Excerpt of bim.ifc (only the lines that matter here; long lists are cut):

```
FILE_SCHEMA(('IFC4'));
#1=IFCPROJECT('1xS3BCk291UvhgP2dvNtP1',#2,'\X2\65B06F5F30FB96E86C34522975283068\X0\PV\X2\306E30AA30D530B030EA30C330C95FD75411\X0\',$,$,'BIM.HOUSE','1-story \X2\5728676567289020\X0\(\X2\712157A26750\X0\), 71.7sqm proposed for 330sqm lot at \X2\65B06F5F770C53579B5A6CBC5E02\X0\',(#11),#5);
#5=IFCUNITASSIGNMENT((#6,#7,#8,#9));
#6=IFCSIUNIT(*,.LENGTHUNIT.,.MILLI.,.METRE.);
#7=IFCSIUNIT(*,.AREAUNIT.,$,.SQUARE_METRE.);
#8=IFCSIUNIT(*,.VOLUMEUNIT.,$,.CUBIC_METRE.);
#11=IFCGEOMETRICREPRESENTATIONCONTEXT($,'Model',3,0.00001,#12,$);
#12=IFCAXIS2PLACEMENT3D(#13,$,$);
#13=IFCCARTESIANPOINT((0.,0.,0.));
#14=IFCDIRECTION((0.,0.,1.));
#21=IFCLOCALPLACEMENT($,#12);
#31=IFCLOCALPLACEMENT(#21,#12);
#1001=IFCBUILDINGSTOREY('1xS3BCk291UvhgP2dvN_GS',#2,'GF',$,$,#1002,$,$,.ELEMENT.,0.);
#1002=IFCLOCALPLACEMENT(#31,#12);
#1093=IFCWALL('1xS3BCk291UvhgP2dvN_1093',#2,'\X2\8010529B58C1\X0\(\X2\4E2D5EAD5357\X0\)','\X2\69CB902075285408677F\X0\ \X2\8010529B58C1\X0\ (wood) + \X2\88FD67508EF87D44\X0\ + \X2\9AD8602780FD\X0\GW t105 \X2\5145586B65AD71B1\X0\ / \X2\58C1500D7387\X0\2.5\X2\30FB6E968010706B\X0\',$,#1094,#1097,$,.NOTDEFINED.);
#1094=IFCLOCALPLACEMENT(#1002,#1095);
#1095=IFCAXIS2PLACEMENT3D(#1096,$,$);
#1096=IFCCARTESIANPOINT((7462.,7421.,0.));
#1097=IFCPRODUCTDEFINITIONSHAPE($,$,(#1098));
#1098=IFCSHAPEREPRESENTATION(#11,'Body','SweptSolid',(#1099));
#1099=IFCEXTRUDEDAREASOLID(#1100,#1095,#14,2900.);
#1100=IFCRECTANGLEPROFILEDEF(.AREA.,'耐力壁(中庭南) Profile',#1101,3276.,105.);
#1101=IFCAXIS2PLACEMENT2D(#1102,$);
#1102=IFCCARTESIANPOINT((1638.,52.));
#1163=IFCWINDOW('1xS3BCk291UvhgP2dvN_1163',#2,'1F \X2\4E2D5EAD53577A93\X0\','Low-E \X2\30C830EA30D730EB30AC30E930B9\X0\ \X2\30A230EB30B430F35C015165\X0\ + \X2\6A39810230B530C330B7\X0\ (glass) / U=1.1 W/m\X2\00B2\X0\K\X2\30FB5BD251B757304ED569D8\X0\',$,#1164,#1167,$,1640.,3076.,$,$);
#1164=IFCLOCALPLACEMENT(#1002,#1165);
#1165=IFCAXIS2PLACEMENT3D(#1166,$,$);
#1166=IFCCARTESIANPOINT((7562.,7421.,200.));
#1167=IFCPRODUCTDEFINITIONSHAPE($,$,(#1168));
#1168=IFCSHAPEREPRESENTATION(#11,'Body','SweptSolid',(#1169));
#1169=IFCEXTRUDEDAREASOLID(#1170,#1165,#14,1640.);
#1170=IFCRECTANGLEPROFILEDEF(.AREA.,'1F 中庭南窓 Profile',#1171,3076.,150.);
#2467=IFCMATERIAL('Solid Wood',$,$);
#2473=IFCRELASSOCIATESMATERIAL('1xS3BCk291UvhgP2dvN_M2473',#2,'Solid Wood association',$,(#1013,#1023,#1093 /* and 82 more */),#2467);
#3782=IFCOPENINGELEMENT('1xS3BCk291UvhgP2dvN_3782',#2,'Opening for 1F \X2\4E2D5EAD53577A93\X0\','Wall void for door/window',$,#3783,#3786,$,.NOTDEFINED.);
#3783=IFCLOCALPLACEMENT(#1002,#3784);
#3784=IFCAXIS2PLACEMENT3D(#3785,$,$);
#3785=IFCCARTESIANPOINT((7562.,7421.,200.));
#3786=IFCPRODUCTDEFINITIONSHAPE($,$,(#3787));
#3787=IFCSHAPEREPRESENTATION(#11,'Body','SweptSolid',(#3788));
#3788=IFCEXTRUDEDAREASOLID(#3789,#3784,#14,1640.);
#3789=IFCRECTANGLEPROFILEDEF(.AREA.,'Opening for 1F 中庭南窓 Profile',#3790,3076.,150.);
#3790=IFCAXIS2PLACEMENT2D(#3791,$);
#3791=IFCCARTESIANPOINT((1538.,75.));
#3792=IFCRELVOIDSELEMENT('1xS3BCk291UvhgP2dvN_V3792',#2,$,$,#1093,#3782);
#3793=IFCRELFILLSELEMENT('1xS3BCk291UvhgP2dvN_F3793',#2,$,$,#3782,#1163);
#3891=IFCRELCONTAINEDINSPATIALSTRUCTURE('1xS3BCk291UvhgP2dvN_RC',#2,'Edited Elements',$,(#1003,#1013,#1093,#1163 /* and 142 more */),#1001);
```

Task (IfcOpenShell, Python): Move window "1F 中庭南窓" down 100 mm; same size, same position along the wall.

```python
import numpy as np
import ifcopenshell
import ifcopenshell.api.geometry
import ifcopenshell.util.placement
import ifcopenshell.util.unit

model = ifcopenshell.open("bim.ifc")
unit_scale = ifcopenshell.util.unit.calculate_unit_scale(model)

window = model.by_guid("1xS3BCk291UvhgP2dvN_1163")
opening = window.FillsVoids[0].RelatingOpeningElement
dz = -100.0

shift = np.array([0.0, 0.0, dz])
# The window is not placed relative to its opening, so move both.
for product in (opening, window):
    matrix = ifcopenshell.util.placement.get_local_placement(product.ObjectPlacement)
    matrix[:3, 3] += shift
    ifcopenshell.api.geometry.edit_object_placement(model, product=product, matrix=matrix, is_si=False)

print(f"moved by {dz * unit_scale:+.3f} m")

model.write("bim-out.ifc")
```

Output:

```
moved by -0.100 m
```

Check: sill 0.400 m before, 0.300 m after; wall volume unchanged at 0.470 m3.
